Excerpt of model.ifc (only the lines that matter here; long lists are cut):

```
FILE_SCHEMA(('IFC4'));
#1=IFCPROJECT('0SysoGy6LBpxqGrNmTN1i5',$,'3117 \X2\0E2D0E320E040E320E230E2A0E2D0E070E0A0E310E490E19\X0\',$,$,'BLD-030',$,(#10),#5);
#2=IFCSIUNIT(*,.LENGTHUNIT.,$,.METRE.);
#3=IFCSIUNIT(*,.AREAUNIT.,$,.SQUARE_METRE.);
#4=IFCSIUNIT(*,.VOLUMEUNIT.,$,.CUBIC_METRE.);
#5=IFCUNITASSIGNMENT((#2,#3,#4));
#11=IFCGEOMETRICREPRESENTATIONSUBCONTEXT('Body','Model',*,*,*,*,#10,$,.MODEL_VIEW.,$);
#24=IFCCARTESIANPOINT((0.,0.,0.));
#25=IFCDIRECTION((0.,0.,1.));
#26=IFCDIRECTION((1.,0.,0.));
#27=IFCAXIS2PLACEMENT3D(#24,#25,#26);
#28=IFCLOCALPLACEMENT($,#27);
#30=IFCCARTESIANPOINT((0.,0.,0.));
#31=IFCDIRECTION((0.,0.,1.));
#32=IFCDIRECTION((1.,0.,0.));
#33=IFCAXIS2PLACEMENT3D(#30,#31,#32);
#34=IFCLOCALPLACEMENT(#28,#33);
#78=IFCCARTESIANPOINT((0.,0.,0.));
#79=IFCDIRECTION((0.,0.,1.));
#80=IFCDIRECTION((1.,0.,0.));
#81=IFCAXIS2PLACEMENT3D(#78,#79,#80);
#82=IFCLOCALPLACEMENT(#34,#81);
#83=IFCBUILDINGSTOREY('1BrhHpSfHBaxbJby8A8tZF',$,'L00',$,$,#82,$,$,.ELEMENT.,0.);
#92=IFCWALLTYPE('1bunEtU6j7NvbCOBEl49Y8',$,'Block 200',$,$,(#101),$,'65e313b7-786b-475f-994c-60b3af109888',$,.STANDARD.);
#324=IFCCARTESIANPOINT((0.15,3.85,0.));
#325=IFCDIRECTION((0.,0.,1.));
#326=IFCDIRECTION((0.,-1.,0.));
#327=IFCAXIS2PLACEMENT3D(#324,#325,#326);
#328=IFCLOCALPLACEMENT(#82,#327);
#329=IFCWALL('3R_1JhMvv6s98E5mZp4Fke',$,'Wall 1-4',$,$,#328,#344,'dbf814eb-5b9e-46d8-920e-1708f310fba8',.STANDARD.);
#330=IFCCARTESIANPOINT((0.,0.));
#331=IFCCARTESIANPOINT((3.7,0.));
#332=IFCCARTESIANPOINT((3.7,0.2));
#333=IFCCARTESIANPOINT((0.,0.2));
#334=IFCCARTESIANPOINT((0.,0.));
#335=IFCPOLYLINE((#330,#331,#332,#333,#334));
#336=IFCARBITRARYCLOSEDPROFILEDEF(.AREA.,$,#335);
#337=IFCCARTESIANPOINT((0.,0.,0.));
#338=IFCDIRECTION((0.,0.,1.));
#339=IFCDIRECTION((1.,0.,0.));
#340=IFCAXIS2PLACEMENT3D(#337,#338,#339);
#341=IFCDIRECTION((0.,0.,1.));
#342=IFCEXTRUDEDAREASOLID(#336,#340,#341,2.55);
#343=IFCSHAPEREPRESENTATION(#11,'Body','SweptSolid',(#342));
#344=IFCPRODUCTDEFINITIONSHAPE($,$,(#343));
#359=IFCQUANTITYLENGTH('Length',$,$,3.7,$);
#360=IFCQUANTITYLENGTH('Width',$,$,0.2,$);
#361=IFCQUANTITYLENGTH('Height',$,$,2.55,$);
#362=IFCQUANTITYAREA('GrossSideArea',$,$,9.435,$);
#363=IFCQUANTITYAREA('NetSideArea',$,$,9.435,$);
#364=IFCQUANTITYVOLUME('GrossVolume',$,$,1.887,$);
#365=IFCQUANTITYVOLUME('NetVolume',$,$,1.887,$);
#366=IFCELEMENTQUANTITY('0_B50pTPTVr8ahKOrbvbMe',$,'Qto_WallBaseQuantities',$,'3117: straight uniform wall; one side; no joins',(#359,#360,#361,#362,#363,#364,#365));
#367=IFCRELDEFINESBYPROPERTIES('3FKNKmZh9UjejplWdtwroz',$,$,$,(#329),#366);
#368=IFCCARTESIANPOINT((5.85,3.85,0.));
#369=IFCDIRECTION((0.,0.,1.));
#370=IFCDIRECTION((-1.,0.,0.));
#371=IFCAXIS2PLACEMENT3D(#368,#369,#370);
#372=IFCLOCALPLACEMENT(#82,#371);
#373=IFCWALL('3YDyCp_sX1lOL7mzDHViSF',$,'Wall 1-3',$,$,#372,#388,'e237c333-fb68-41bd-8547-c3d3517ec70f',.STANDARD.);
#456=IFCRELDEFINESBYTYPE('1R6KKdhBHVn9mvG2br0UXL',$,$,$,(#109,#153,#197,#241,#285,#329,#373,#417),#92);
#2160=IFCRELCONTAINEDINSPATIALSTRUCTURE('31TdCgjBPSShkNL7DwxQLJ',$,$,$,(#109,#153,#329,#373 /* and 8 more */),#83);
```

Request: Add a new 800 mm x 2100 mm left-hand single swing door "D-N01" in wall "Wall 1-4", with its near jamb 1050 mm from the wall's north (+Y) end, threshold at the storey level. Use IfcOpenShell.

```python
import numpy as np
import ifcopenshell
import ifcopenshell.api.feature
import ifcopenshell.api.geometry
import ifcopenshell.api.pset
import ifcopenshell.api.root
import ifcopenshell.api.spatial
import ifcopenshell.geom
import ifcopenshell.util.element
import ifcopenshell.util.placement
import ifcopenshell.util.representation
import ifcopenshell.util.shape
import ifcopenshell.util.unit

model = ifcopenshell.open("model.ifc")
unit_scale = ifcopenshell.util.unit.calculate_unit_scale(model)
area_scale = ifcopenshell.util.unit.calculate_unit_scale(model, "AREAUNIT")
volume_scale = ifcopenshell.util.unit.calculate_unit_scale(model, "VOLUMEUNIT")
settings = ifcopenshell.geom.settings()


def volume(element):
    """Net volume in cubic metres, openings subtracted."""
    shape = ifcopenshell.geom.create_shape(settings, element)
    return ifcopenshell.util.shape.get_volume(shape.geometry)


wall = model.by_guid("3R_1JhMvv6s98E5mZp4Fke")
storey = ifcopenshell.util.element.get_container(wall, ifc_class="IfcBuildingStorey")
context = ifcopenshell.util.representation.get_context(model, "Model", "Body", "MODEL_VIEW")
before = volume(wall)

width, height, from_end, sill = 0.8, 2.1, 1.05, 0.0  # metres

# The wall runs along its own X axis, and the end named is its -X end.
wall_shape = ifcopenshell.geom.create_shape(settings, wall)
x, y, z = ifcopenshell.util.shape.get_vertices(wall_shape.geometry).T
start = x.min() + from_end
face, thickness = float(y.min()), float(y.max() - y.min())
wall_matrix = ifcopenshell.util.placement.get_local_placement(wall.ObjectPlacement)
level = ifcopenshell.util.placement.get_local_placement(storey.ObjectPlacement)[2, 3]


def in_wall(x, y):
    """Placement at x, y metres in the wall's axes, at sill height."""
    matrix = wall_matrix.copy()
    matrix[:, 3] = wall_matrix @ np.array([x / unit_scale, y / unit_scale, 0.0, 1.0])
    matrix[2, 3] = level + sill / unit_scale
    return matrix


# Opening: a box that overshoots both wall faces by 50 mm.
opening = ifcopenshell.api.root.create_entity(model, ifc_class="IfcOpeningElement", predefined_type="OPENING")
box = ifcopenshell.api.geometry.add_wall_representation(
    model, context=context, length=width, height=height, thickness=thickness + 0.1
)
ifcopenshell.api.geometry.assign_representation(model, product=opening, representation=box)
ifcopenshell.api.geometry.edit_object_placement(model, product=opening, matrix=in_wall(start, face - 0.05), is_si=False)
ifcopenshell.api.feature.add_feature(model, feature=opening, element=wall)

door = ifcopenshell.api.root.create_entity(model, ifc_class="IfcDoor", name="D-N01", predefined_type="DOOR")
door.OverallWidth, door.OverallHeight = width / unit_scale, height / unit_scale
door.OperationType = "SINGLE_SWING_LEFT"
body = ifcopenshell.api.geometry.add_door_representation(
    model,
    context=context,
    overall_width=door.OverallWidth,
    overall_height=door.OverallHeight,
    operation_type="SINGLE_SWING_LEFT",
    lining_properties={"LiningDepth": thickness / unit_scale, "ThresholdDepth": thickness / unit_scale},
)
ifcopenshell.api.geometry.assign_representation(model, product=door, representation=body)
ifcopenshell.api.spatial.assign_container(model, products=[door], relating_structure=storey)
ifcopenshell.api.feature.add_filling(model, opening=opening, element=door)

# The lining spans the wall, so the door starts at the wall face.
ifcopenshell.api.geometry.edit_object_placement(model, product=door, matrix=in_wall(start, face), is_si=False)

after = volume(wall)

# Update the wall's stored quantities.
qto = model.by_id(ifcopenshell.util.element.get_pset(wall, "Qto_WallBaseQuantities", should_inherit=False)["id"])
ifcopenshell.api.pset.edit_qto(model, qto=qto, properties={
    "NetSideArea": after / thickness / area_scale,
    "NetVolume": after / volume_scale,
})

print(f"wall volume {before:.3f} -> {after:.3f} m3")

model.write("model_v2.ifc")
```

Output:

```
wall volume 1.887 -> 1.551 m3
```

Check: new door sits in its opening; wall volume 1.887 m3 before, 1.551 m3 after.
